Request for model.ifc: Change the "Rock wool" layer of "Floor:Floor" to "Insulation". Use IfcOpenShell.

First a look at what the model holds.

```python
import ifcopenshell
import ifcopenshell.util.element

model = ifcopenshell.open("model.ifc")
print(model.schema)
for layer_set in model.by_type("IfcMaterialLayerSet"):
    if layer_set.LayerSetName == "Floor:Floor":
        for layer in layer_set.MaterialLayers:
            print(layer.id(), layer.Material and layer.Material.Name, layer.LayerThickness, sep=" | ")
        print(len(ifcopenshell.util.element.get_elements_by_material(model, layer_set)), "elements and types use it")
print(sorted(m.Name for m in model.by_type("IfcMaterial") if m.Name)[:60])
```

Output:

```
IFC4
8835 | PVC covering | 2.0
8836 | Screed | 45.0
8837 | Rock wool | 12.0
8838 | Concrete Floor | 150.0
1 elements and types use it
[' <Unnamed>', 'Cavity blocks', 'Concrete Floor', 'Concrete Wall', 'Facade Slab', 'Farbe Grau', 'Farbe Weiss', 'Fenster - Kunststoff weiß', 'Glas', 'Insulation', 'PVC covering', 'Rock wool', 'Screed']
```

```python
import ifcopenshell
import ifcopenshell.api.material

model = ifcopenshell.open("model.ifc")

layer_set = next(s for s in model.by_type("IfcMaterialLayerSet") if s.LayerSetName == "Floor:Floor")
layer = next(l for l in layer_set.MaterialLayers if l.Material and l.Material.Name == "Rock wool")
material = next(m for m in model.by_type("IfcMaterial") if m.Name == "Insulation")

# Point this one layer at the other material; renaming the old one would change it everywhere.
ifcopenshell.api.material.edit_layer(model, layer=layer, attributes={}, material=material)

print([l.Material.Name if l.Material else None for l in layer_set.MaterialLayers])

model.write("model_edited.ifc")
```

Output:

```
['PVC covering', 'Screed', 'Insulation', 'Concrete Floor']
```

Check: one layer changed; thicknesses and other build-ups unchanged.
